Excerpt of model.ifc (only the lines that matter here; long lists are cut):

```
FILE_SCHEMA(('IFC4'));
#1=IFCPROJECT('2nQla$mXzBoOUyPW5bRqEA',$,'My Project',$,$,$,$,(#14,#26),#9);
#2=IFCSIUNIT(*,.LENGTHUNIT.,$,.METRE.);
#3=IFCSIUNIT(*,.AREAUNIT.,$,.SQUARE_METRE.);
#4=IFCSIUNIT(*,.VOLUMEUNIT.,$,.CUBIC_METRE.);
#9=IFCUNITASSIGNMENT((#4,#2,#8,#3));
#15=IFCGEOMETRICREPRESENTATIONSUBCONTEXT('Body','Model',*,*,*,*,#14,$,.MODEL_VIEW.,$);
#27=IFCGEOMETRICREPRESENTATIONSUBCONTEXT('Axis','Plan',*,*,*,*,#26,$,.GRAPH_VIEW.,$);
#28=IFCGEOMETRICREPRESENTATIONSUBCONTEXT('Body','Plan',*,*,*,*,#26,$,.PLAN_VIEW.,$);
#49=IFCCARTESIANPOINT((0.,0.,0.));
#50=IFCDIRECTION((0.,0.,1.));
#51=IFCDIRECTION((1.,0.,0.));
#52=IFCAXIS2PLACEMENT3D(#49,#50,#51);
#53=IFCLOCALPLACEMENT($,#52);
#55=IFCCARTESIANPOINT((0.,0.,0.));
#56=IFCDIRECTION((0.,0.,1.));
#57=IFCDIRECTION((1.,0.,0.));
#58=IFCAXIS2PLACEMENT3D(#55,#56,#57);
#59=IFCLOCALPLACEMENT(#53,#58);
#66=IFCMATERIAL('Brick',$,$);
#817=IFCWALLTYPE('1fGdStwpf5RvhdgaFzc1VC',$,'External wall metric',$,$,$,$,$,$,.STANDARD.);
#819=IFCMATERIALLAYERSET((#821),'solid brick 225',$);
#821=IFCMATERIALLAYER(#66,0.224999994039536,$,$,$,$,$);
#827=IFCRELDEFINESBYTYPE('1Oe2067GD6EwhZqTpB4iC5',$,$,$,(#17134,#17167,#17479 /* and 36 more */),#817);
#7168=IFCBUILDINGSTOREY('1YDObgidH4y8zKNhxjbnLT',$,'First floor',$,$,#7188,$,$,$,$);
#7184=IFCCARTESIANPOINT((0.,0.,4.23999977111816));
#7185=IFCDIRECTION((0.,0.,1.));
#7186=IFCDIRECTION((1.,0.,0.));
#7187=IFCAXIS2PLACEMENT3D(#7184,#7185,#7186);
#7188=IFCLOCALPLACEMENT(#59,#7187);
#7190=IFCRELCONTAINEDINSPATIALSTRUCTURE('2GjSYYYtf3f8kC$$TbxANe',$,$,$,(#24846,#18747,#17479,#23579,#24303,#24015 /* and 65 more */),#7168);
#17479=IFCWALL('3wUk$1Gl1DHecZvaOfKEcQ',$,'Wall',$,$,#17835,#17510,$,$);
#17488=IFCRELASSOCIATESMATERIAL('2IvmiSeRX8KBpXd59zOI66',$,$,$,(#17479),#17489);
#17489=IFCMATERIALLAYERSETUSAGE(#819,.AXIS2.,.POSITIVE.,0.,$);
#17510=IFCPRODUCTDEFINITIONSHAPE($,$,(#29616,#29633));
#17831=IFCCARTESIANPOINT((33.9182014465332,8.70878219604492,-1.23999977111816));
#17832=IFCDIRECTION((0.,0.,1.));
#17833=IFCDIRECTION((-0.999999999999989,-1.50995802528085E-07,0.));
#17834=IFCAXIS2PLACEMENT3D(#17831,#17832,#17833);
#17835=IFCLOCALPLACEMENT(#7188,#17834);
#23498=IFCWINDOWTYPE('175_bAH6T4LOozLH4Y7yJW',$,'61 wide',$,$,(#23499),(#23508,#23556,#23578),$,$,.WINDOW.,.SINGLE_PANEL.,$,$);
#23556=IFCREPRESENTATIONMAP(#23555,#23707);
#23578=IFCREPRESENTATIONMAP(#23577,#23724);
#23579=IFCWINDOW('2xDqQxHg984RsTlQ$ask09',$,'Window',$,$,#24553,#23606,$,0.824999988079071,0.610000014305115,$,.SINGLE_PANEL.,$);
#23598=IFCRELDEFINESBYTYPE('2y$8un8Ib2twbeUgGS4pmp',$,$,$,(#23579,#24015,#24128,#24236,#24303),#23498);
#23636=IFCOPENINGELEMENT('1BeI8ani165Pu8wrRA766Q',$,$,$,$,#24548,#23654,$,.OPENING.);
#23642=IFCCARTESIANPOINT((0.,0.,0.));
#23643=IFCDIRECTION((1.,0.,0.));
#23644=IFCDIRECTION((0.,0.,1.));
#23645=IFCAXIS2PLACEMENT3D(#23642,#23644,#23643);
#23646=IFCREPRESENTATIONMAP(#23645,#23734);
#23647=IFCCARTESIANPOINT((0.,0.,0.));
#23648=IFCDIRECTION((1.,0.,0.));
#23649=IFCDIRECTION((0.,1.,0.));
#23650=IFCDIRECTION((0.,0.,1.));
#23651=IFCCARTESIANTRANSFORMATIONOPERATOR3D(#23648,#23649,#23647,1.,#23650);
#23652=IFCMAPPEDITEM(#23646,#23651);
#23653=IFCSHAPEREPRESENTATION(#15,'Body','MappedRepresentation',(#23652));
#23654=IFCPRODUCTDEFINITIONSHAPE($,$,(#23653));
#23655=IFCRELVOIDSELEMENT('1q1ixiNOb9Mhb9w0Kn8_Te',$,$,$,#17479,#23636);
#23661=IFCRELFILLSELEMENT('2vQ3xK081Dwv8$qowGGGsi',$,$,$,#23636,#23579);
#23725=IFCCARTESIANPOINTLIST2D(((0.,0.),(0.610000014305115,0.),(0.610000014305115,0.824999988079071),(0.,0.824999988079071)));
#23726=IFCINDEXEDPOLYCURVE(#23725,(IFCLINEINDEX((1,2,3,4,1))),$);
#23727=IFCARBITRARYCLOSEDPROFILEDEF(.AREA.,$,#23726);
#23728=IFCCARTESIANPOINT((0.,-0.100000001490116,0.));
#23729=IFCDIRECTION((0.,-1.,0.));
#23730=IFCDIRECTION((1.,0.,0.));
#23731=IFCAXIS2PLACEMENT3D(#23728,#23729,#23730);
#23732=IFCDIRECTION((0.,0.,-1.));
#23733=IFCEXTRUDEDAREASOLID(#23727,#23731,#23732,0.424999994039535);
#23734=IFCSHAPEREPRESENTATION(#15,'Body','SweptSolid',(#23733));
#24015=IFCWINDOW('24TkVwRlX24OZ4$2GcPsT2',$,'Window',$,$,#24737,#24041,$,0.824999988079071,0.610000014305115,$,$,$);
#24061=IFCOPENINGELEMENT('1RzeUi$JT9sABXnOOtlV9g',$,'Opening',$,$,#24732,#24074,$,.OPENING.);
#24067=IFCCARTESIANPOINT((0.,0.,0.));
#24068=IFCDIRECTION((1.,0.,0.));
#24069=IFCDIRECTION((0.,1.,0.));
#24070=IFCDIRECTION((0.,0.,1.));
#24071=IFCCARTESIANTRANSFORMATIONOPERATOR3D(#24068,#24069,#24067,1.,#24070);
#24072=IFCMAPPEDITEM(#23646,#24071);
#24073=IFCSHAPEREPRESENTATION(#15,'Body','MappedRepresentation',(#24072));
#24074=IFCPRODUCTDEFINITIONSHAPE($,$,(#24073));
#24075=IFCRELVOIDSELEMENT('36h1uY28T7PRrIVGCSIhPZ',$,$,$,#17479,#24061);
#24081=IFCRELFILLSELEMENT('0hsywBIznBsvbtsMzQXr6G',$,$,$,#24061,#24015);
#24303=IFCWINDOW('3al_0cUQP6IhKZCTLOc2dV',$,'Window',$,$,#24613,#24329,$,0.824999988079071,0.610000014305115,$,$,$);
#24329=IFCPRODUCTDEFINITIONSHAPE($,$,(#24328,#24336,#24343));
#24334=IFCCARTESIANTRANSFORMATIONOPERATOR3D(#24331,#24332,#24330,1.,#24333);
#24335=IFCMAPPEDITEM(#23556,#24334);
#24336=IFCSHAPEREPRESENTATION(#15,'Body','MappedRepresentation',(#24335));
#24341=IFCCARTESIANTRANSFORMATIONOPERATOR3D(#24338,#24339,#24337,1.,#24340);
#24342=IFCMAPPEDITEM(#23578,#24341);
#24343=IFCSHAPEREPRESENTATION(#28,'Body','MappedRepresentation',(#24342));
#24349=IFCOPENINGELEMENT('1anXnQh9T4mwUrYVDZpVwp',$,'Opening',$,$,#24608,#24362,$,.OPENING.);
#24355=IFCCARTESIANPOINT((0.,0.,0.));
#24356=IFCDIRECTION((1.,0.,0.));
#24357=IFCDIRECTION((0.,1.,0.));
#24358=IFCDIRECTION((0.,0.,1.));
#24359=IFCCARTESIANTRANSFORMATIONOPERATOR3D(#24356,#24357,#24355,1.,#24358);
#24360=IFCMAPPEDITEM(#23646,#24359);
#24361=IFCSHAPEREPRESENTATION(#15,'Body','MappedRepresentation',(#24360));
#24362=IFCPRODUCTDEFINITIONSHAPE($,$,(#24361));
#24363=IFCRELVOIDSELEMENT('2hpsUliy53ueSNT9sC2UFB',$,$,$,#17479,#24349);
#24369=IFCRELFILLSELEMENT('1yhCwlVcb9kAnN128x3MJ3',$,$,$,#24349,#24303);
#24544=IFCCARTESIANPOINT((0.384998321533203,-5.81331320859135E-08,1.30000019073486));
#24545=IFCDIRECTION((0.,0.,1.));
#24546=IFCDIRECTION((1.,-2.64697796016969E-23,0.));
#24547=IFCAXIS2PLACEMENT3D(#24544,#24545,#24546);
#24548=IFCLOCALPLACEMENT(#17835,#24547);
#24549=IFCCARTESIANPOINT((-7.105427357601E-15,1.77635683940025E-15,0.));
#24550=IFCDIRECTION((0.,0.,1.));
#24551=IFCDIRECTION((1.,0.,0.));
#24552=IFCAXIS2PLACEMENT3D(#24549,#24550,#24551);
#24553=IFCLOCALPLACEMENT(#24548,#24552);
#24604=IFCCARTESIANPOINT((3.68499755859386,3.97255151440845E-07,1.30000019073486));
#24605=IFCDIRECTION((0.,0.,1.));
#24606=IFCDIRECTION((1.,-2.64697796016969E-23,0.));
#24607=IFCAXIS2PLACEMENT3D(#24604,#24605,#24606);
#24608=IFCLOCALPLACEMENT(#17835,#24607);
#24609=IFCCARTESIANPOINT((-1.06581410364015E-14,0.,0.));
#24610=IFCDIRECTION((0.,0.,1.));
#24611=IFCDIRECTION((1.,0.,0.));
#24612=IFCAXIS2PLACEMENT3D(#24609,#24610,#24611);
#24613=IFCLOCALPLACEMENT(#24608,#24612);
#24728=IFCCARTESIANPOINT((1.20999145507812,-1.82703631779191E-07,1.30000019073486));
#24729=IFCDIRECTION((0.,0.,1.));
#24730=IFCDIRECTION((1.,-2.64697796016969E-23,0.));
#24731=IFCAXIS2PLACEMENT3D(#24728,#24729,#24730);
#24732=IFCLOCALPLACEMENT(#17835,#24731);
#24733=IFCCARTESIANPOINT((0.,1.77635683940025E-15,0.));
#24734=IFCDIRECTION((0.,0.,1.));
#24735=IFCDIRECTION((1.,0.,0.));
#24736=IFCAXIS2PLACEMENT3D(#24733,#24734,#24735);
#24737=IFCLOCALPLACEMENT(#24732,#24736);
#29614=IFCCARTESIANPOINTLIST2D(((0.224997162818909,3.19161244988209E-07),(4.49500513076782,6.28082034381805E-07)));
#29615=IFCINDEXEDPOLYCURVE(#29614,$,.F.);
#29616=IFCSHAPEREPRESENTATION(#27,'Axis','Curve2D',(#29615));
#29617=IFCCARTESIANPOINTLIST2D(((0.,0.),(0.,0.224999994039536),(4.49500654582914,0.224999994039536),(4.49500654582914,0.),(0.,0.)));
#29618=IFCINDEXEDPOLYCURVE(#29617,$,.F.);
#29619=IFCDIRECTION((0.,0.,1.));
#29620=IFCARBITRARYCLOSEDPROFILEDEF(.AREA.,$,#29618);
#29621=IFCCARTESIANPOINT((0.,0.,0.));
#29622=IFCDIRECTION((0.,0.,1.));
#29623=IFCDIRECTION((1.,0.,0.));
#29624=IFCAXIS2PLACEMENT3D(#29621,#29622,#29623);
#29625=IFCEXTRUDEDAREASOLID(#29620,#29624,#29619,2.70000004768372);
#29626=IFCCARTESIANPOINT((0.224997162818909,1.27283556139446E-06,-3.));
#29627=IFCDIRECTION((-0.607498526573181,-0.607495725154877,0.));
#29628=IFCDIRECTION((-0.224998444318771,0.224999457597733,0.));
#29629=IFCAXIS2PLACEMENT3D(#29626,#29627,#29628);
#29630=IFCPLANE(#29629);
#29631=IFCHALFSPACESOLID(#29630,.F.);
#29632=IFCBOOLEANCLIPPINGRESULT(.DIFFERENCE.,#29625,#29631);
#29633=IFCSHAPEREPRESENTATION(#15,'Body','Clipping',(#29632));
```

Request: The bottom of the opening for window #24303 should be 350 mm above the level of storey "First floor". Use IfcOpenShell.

```python
import numpy as np
import ifcopenshell
import ifcopenshell.api.geometry
import ifcopenshell.geom
import ifcopenshell.util.element
import ifcopenshell.util.placement
import ifcopenshell.util.shape
import ifcopenshell.util.unit

model = ifcopenshell.open("model.ifc")
unit_scale = ifcopenshell.util.unit.calculate_unit_scale(model)

window = model.by_id(24303)
opening = window.FillsVoids[0].RelatingOpeningElement
storey = ifcopenshell.util.element.get_container(window, ifc_class="IfcBuildingStorey")
level = ifcopenshell.util.placement.get_local_placement(storey.ObjectPlacement)[2, 3]

# The opening's origin need not be at the sill, so measure its lowest point.
shape = ifcopenshell.geom.create_shape(ifcopenshell.geom.settings(), opening)
bottom = ifcopenshell.util.shape.get_shape_bottom_elevation(shape, shape.geometry) / unit_scale
dz = level + 0.35 - bottom

shift = np.array([0.0, 0.0, dz])
# The window is placed relative to its opening, so it follows when the opening moves.
matrix = ifcopenshell.util.placement.get_local_placement(opening.ObjectPlacement)
matrix[:3, 3] += shift
ifcopenshell.api.geometry.edit_object_placement(
    model, product=opening, matrix=matrix, is_si=False, should_transform_children=True
)

print(f"moved by {dz * unit_scale:+.3f} m")

model.write("model_rev.ifc")
```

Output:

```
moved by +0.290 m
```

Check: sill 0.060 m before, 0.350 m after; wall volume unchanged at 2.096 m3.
